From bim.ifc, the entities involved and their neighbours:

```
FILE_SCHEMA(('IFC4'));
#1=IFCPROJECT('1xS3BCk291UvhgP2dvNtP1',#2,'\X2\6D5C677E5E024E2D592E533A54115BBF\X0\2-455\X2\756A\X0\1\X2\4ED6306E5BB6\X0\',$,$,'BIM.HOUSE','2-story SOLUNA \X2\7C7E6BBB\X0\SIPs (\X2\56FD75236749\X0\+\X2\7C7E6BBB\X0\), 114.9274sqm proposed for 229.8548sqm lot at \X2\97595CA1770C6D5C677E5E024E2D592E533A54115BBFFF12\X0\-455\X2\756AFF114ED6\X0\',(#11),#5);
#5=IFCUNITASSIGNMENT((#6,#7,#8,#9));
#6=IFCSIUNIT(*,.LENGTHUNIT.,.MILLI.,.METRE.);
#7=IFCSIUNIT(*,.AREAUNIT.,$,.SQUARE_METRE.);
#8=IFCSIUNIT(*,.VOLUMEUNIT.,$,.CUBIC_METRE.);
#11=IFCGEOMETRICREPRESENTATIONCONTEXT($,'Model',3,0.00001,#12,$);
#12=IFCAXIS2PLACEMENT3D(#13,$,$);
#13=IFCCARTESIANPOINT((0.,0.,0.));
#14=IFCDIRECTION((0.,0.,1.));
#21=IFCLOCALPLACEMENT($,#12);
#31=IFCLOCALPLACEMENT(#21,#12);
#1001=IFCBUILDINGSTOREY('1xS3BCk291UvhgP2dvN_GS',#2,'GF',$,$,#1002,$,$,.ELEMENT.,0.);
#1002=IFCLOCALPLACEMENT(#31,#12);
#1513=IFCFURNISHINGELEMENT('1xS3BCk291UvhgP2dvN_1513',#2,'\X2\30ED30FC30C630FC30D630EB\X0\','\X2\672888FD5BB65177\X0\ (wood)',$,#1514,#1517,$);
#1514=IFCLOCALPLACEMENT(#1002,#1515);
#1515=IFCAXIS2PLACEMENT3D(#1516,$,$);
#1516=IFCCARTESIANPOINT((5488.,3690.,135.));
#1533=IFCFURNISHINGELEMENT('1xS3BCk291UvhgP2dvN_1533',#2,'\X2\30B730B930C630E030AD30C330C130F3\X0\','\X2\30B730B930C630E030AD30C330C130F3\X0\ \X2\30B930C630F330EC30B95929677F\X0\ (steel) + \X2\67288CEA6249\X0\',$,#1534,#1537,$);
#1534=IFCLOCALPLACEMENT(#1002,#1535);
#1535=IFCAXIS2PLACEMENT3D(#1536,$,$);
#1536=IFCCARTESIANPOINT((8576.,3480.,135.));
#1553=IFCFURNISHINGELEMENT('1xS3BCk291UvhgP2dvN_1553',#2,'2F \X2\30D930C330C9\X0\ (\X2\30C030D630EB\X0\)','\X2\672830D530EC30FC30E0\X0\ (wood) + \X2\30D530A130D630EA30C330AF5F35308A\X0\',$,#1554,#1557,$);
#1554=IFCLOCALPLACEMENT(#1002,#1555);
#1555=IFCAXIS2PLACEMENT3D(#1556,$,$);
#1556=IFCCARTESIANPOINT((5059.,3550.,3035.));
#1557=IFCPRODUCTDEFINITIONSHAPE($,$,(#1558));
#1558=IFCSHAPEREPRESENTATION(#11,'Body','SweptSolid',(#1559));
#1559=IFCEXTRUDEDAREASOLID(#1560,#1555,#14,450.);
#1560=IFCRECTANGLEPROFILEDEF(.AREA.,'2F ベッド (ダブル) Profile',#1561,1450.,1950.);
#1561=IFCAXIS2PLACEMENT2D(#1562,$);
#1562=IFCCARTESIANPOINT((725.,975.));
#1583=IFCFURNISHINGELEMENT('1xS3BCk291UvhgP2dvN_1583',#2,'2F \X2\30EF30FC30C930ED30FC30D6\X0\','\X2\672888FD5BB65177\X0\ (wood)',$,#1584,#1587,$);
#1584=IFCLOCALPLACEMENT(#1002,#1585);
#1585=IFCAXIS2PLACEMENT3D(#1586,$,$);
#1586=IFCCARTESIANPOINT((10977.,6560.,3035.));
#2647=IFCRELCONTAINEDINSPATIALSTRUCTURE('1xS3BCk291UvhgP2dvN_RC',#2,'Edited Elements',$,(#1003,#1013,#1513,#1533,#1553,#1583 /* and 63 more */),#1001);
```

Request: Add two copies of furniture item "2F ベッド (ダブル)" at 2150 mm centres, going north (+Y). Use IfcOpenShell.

```python
import numpy as np
import ifcopenshell
import ifcopenshell.api.geometry
import ifcopenshell.api.root
import ifcopenshell.util.element
import ifcopenshell.util.placement

model = ifcopenshell.open("bim.ifc")


def reuse_history(source, copy):
    """copy_class also copies each property set's owner history, people and application; keep the originals."""
    for rel in copy.IsDefinedBy:
        if rel.is_a("IfcRelDefinesByProperties") and (history := rel.RelatingPropertyDefinition.OwnerHistory):
            rel.RelatingPropertyDefinition.OwnerHistory = source.OwnerHistory
            ifcopenshell.util.element.remove_deep2(model, history)


source = model.by_guid("1xS3BCk291UvhgP2dvN_1553")
base = ifcopenshell.util.placement.get_local_placement(source.ObjectPlacement)
step = np.array([0.0, 1.0, 0.0]) * 2150.0

for i in range(1, 3):
    copy = ifcopenshell.api.root.copy_class(model, product=source)
    copy.Representation = ifcopenshell.util.element.copy_deep(
        model, source.Representation, exclude=["IfcGeometricRepresentationContext", "IfcRepresentationMap"]
    )
    reuse_history(source, copy)
    matrix = base.copy()
    matrix[:3, 3] += i * step
    print("added at", matrix[:3, 3].round(3) + 0.0)
    ifcopenshell.api.geometry.edit_object_placement(model, product=copy, matrix=matrix, is_si=False)

model.write("bim_updated.ifc")
```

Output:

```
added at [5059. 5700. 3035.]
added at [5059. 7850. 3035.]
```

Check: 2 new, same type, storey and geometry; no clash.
